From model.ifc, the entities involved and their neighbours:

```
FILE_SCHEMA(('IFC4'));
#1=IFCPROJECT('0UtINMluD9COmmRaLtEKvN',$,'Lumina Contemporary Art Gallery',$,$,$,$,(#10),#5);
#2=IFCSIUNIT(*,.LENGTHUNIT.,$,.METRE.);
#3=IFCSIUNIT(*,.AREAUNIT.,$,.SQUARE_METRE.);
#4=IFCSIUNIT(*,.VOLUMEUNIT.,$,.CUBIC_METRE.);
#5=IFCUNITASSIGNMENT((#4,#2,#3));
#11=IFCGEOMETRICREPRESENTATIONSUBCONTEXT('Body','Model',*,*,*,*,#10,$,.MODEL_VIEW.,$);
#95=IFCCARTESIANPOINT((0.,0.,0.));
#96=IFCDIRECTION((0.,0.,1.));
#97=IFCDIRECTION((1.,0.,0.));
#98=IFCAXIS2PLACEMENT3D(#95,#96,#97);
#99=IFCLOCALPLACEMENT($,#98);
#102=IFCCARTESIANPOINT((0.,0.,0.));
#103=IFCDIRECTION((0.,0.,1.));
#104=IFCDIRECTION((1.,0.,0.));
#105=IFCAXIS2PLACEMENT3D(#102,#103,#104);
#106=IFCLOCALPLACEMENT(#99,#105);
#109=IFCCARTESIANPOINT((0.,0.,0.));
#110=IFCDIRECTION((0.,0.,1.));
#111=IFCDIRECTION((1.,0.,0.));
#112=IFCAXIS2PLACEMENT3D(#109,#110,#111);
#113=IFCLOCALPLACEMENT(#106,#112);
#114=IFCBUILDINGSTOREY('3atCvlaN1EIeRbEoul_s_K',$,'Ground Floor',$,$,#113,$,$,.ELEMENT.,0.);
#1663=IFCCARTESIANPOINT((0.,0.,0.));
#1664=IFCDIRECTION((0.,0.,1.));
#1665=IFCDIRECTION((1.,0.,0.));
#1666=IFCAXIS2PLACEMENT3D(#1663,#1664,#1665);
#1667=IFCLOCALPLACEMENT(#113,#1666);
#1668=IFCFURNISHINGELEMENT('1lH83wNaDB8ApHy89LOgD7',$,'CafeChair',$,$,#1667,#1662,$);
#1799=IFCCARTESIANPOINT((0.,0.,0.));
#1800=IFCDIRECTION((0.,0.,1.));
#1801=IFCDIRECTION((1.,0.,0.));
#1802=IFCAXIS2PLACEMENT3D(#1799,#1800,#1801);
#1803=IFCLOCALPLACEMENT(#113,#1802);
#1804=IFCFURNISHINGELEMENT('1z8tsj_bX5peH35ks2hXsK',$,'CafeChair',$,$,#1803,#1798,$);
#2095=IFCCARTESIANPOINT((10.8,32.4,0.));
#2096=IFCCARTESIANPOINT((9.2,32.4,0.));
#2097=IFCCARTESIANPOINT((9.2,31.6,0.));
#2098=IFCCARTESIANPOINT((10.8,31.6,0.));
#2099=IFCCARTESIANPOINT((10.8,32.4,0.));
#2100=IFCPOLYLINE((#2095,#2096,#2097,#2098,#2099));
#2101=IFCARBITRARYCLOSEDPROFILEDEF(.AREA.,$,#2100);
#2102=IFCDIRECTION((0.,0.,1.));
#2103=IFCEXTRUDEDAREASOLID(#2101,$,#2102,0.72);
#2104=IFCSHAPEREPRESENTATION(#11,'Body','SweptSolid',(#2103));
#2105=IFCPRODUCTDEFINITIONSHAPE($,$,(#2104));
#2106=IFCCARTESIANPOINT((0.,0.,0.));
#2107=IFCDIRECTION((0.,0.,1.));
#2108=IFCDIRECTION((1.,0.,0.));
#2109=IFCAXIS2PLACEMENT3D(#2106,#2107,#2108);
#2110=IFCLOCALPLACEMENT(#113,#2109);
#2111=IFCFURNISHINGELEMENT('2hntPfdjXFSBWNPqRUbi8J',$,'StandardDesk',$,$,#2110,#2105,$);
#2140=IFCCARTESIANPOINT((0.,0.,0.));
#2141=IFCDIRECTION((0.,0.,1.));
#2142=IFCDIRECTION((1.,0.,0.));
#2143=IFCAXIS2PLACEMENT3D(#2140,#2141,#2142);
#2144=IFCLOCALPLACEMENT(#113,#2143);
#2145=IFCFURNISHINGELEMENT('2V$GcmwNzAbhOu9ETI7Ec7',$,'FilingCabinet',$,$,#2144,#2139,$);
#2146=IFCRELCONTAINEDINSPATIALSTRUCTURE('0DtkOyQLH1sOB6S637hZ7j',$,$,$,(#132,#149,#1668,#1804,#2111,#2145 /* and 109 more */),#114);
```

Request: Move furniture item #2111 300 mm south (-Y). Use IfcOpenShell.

```python
import ifcopenshell
import ifcopenshell.api.geometry
import ifcopenshell.util.placement

model = ifcopenshell.open("model.ifc")

item = model.by_guid("2hntPfdjXFSBWNPqRUbi8J")
matrix = ifcopenshell.util.placement.get_local_placement(item.ObjectPlacement)
matrix[1, 3] -= 0.3
ifcopenshell.api.geometry.edit_object_placement(model, product=item, matrix=matrix, is_si=False)

print(ifcopenshell.util.placement.get_local_placement(item.ObjectPlacement).round(3) + 0.0)

model.write("model-out.ifc")
```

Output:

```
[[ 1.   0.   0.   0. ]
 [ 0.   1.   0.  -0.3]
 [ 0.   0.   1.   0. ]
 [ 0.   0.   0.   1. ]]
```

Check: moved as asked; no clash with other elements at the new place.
